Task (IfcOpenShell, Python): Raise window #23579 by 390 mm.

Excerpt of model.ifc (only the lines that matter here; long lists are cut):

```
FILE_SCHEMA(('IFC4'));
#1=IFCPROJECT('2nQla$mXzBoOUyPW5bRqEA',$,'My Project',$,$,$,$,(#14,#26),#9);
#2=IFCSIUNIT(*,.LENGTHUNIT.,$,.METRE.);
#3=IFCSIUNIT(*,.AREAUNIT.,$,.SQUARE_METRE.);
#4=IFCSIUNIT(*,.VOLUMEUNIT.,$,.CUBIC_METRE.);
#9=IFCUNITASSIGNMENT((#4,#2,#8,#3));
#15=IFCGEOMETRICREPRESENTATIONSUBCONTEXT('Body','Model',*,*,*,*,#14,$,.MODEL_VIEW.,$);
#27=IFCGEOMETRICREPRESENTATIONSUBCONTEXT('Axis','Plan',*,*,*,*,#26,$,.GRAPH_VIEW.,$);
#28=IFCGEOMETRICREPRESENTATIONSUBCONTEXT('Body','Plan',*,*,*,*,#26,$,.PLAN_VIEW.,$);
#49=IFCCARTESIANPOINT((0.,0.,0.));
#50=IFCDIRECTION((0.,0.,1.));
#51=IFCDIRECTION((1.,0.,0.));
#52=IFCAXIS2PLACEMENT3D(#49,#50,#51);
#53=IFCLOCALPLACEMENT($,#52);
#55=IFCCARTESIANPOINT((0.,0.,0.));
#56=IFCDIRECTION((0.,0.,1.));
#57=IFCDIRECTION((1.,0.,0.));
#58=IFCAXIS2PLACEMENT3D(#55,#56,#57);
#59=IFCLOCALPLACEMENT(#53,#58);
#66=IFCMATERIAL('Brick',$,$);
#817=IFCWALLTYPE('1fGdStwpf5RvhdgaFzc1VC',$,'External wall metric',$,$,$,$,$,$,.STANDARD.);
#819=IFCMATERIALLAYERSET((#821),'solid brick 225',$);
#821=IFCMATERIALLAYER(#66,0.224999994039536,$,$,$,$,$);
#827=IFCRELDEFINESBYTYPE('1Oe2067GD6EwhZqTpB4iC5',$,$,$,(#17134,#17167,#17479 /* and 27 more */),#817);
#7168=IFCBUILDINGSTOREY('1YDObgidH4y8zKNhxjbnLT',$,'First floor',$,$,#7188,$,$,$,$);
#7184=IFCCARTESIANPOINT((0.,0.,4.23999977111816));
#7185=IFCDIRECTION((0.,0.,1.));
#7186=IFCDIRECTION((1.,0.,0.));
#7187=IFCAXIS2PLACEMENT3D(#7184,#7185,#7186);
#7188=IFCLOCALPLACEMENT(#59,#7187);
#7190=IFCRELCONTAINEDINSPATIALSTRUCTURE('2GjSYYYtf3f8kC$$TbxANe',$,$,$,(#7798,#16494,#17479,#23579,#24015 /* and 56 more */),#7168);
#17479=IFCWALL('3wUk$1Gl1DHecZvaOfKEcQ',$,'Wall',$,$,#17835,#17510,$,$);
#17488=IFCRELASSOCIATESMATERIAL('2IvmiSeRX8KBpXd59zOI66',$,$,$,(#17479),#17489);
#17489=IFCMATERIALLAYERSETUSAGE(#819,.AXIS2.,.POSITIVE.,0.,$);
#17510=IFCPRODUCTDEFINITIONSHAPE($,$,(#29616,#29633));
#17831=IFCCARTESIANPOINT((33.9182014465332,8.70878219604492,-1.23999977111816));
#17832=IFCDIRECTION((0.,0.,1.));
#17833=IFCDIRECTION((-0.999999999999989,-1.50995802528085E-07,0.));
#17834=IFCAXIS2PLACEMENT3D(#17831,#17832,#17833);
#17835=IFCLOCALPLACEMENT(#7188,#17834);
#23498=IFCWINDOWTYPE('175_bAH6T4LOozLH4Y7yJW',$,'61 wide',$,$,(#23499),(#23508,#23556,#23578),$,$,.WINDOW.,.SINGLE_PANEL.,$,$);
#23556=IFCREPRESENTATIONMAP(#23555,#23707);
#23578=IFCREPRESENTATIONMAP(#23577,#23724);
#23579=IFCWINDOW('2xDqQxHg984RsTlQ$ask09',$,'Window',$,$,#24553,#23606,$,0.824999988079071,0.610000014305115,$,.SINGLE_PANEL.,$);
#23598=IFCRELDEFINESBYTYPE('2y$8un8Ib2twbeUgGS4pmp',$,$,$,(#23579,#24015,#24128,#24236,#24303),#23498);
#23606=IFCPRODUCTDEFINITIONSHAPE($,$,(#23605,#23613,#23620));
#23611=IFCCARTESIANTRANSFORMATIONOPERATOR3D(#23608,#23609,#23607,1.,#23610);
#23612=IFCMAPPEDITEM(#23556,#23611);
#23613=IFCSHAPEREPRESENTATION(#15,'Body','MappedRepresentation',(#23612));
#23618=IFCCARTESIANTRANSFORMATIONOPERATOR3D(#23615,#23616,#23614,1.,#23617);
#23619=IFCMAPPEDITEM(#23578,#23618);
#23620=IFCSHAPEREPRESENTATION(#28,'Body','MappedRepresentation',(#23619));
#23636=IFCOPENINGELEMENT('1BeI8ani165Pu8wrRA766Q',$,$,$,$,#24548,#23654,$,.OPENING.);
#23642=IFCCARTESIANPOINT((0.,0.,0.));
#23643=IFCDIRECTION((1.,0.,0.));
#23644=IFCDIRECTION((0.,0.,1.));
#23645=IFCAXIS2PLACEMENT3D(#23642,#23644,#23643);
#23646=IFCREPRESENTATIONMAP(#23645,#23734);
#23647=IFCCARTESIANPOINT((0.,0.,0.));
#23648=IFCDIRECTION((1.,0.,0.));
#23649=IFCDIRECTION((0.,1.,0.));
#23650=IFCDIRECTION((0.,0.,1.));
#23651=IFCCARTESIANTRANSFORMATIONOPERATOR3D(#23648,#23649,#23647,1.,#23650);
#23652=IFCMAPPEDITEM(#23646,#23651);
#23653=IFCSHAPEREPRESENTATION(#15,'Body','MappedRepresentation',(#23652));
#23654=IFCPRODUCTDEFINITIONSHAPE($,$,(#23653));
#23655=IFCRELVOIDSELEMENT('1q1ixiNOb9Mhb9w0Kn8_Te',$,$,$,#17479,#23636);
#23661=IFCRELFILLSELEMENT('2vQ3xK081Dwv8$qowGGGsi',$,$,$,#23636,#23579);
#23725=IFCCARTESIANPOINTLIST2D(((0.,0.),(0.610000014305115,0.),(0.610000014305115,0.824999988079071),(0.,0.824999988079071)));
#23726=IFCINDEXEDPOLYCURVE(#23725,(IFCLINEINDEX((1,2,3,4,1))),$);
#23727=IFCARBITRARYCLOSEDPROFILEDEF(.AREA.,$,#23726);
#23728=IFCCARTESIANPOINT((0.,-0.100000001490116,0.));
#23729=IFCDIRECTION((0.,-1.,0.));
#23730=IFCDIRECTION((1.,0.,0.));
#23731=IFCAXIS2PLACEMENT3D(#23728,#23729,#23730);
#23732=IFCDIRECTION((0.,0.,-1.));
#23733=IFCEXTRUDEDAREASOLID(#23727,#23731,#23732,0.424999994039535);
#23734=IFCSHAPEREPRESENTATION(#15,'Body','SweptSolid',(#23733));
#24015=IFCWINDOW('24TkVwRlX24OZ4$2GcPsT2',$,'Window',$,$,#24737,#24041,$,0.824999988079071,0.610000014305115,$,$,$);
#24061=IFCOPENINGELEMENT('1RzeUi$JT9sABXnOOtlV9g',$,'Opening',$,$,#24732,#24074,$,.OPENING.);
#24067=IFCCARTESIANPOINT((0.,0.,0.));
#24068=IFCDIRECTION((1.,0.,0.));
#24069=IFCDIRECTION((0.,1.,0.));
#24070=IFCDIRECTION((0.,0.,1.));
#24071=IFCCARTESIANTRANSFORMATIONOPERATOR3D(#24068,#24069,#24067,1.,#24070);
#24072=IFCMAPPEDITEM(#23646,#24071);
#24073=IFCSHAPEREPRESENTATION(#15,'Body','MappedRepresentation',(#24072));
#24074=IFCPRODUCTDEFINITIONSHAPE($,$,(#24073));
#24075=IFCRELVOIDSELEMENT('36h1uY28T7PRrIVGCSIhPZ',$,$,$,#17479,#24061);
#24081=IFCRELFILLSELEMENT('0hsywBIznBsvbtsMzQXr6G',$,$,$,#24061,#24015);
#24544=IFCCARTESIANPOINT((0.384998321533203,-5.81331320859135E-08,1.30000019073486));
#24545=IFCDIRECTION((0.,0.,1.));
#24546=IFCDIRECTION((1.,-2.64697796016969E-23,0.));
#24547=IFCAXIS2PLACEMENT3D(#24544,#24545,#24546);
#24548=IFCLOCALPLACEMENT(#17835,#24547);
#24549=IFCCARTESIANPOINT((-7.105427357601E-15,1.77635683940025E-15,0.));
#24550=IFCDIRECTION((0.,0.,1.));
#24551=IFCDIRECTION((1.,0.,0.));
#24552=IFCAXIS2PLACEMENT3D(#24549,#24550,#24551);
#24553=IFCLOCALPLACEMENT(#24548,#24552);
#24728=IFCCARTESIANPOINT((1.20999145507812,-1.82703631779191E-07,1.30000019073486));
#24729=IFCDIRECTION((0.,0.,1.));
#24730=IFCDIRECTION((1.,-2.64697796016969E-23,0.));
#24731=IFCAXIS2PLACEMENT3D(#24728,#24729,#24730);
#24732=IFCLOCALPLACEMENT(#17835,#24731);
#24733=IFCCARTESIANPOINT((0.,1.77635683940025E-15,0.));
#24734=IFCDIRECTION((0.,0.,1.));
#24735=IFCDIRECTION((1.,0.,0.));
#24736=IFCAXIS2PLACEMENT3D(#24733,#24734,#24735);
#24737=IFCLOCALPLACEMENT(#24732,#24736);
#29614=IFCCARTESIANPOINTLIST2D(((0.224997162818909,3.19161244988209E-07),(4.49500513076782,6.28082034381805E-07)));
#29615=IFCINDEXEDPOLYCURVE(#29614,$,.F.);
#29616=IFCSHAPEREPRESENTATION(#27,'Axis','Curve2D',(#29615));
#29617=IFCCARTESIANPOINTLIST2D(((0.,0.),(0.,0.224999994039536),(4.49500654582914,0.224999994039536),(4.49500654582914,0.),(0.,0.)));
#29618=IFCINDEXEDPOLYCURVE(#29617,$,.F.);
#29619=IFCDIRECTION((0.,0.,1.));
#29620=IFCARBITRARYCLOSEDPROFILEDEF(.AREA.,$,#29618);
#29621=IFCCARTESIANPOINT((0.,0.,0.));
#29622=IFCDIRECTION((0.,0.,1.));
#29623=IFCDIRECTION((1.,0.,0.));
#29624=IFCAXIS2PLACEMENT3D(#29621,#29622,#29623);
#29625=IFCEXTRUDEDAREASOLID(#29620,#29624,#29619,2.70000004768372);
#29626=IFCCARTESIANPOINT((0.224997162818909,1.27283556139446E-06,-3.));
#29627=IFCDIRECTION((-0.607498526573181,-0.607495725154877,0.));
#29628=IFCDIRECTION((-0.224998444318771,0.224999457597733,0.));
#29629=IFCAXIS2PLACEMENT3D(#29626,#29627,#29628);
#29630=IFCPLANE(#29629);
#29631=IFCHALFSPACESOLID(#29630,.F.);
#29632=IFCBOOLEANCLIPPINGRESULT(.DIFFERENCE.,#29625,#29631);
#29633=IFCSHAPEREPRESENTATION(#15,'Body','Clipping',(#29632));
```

```python
import numpy as np
import ifcopenshell
import ifcopenshell.api.geometry
import ifcopenshell.util.placement
import ifcopenshell.util.unit

model = ifcopenshell.open("model.ifc")
unit_scale = ifcopenshell.util.unit.calculate_unit_scale(model)

window = model.by_id(23579)
opening = window.FillsVoids[0].RelatingOpeningElement
dz = 0.39

shift = np.array([0.0, 0.0, dz])
# The window is placed relative to its opening, so it follows when the opening moves.
matrix = ifcopenshell.util.placement.get_local_placement(opening.ObjectPlacement)
matrix[:3, 3] += shift
ifcopenshell.api.geometry.edit_object_placement(
    model, product=opening, matrix=matrix, is_si=False, should_transform_children=True
)

print(f"moved by {dz * unit_scale:+.3f} m")

model.write("model_rev.ifc")
```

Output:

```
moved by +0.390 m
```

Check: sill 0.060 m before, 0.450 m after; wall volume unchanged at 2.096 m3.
